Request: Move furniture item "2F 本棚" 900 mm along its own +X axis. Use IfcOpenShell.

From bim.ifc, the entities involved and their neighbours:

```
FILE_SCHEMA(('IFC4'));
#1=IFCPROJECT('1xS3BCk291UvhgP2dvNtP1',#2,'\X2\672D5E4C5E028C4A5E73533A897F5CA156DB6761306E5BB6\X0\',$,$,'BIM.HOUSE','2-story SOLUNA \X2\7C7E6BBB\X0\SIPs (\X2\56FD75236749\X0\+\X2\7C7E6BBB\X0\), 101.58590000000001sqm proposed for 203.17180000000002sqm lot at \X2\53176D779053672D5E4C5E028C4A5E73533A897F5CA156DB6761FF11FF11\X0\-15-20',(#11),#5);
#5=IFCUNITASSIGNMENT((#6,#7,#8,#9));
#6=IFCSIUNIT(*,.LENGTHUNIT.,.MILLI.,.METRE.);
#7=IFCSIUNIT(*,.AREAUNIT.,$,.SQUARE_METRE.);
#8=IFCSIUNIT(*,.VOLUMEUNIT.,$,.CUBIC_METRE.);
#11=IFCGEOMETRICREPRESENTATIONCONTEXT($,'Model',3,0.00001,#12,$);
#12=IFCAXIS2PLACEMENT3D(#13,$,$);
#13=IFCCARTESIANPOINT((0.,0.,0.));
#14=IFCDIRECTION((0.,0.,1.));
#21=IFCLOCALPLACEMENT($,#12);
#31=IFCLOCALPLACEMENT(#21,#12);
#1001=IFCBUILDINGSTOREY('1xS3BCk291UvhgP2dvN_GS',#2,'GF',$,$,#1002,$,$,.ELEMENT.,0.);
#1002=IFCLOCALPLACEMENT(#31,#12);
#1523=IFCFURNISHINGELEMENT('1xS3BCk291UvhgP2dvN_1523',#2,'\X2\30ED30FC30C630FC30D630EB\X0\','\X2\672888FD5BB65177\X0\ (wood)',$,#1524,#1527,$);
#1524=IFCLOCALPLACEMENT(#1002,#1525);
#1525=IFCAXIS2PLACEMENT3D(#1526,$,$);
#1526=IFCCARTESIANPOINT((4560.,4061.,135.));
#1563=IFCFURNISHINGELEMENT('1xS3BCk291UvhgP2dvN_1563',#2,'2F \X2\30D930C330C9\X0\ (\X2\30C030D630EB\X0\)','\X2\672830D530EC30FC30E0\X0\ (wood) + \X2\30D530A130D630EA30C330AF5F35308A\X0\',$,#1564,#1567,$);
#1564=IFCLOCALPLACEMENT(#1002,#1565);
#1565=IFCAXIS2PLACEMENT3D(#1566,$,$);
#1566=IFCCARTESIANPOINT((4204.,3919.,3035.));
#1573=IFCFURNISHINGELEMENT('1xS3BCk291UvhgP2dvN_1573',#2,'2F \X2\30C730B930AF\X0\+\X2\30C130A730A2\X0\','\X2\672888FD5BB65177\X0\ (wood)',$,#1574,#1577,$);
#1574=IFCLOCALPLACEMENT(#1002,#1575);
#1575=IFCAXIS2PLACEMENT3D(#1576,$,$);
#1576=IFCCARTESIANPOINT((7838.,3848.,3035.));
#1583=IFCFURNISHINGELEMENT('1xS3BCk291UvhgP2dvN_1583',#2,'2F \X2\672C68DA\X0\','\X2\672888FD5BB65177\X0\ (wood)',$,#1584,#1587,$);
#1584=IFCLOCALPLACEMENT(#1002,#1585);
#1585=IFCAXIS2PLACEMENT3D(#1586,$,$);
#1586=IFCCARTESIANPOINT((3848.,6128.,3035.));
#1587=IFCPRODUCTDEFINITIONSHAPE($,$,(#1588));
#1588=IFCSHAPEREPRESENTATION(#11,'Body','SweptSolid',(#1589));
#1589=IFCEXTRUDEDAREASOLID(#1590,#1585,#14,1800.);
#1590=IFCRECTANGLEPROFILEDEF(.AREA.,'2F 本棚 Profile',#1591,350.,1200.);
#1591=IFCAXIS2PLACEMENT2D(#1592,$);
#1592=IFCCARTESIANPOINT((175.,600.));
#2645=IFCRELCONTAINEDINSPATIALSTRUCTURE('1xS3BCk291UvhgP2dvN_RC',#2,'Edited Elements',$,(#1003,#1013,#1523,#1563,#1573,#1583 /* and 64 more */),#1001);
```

```python
import ifcopenshell
import ifcopenshell.api.geometry
import ifcopenshell.util.placement
import ifcopenshell.util.unit

model = ifcopenshell.open("bim.ifc")
unit_scale = ifcopenshell.util.unit.calculate_unit_scale(model)

item = model.by_guid("1xS3BCk291UvhgP2dvN_1583")
matrix = ifcopenshell.util.placement.get_local_placement(item.ObjectPlacement)
matrix[:3, 3] += matrix[:3, 0] * 0.9 / unit_scale
ifcopenshell.api.geometry.edit_object_placement(model, product=item, matrix=matrix, is_si=False)

print(ifcopenshell.util.placement.get_local_placement(item.ObjectPlacement).round(3) + 0.0)

model.write("bim_v2.ifc")
```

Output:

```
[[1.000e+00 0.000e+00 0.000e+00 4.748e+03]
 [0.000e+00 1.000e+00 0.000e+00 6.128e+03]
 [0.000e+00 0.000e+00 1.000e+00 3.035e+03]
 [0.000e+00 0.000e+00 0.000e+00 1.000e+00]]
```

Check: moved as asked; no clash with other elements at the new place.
